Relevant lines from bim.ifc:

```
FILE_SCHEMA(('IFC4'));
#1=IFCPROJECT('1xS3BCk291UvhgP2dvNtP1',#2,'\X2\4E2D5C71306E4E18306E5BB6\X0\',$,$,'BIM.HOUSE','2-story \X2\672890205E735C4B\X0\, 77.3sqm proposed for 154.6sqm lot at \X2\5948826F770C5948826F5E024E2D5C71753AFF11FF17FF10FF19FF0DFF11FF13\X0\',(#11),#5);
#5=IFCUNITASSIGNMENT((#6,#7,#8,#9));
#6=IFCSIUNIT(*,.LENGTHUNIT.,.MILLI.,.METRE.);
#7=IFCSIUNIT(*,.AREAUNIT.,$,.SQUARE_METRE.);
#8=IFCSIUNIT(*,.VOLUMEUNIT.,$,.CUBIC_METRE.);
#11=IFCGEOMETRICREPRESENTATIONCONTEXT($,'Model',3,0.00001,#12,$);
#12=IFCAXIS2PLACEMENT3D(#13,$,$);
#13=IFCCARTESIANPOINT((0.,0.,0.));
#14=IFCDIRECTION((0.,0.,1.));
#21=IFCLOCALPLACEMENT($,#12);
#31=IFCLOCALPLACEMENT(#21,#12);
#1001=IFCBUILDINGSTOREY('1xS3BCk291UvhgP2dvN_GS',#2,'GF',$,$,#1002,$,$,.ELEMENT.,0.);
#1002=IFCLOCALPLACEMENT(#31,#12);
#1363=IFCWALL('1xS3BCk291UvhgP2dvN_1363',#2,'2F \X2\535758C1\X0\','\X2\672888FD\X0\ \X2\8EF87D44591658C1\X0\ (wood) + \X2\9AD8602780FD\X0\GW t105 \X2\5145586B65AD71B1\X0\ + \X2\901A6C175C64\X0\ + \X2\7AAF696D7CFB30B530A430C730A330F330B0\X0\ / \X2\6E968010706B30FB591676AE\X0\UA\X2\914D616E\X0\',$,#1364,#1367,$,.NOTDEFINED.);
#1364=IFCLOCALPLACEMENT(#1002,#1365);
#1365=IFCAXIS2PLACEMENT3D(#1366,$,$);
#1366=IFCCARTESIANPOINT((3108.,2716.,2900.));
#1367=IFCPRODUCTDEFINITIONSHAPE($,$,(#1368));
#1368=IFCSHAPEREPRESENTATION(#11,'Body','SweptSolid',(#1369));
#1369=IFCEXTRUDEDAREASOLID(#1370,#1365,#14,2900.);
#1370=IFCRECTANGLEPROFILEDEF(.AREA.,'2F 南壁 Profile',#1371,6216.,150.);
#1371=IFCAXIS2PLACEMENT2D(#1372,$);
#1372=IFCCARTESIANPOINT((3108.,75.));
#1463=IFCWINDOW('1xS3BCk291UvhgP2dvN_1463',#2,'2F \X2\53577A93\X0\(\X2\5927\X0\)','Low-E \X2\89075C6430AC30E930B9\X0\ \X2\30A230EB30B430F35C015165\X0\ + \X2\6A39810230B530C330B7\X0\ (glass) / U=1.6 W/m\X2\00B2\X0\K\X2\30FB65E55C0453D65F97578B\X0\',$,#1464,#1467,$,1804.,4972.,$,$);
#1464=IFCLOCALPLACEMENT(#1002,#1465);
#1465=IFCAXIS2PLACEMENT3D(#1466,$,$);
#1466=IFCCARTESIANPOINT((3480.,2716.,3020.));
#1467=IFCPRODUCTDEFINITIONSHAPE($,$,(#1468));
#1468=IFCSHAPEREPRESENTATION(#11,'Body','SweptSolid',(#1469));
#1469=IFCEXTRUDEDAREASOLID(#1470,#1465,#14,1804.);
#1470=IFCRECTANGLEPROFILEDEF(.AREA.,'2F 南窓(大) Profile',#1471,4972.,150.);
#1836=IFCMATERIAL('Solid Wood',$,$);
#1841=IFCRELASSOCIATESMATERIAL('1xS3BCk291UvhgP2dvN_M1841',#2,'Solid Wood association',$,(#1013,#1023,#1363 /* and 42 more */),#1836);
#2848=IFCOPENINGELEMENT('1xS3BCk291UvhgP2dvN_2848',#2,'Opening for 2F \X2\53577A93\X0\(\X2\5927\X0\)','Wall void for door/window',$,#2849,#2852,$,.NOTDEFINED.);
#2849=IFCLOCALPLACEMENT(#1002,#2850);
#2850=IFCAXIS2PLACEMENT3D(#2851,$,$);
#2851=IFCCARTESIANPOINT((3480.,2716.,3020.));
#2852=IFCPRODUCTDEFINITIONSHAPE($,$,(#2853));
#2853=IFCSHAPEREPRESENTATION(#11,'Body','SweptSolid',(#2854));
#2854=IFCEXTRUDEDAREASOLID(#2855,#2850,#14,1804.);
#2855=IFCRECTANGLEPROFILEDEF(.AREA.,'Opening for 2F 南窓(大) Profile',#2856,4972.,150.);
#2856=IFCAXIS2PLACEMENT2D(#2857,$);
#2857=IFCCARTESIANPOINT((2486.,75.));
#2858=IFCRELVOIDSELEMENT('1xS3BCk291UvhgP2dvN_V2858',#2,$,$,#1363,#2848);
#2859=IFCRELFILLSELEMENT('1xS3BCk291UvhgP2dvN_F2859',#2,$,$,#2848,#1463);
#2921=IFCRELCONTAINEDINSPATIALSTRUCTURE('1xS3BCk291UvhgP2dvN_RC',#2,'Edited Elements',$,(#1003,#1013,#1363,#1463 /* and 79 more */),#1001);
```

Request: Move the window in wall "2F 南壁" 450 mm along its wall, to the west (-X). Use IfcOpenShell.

```python
import ifcopenshell
import ifcopenshell.api.geometry
import ifcopenshell.util.placement

model = ifcopenshell.open("bim.ifc")

window = model.by_guid("1xS3BCk291UvhgP2dvN_1463")
opening = window.FillsVoids[0].RelatingOpeningElement
wall = opening.VoidsElements[0].RelatingBuildingElement

wall_matrix = ifcopenshell.util.placement.get_local_placement(wall.ObjectPlacement)
shift = wall_matrix[:3, 0] * -450.0
before = ifcopenshell.util.placement.get_local_placement(window.ObjectPlacement)[:3, 3].copy()

# The window is not placed relative to its opening, so move both.
for product in (opening, window):
    matrix = ifcopenshell.util.placement.get_local_placement(product.ObjectPlacement)
    matrix[:3, 3] += shift
    ifcopenshell.api.geometry.edit_object_placement(model, product=product, matrix=matrix, is_si=False)

after = ifcopenshell.util.placement.get_local_placement(window.ObjectPlacement)[:3, 3]
print("window moved by", (after - before).round(3) + 0.0)

model.write("bim_edited.ifc")
```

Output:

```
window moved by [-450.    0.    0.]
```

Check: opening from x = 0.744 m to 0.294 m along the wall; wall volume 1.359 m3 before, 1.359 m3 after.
